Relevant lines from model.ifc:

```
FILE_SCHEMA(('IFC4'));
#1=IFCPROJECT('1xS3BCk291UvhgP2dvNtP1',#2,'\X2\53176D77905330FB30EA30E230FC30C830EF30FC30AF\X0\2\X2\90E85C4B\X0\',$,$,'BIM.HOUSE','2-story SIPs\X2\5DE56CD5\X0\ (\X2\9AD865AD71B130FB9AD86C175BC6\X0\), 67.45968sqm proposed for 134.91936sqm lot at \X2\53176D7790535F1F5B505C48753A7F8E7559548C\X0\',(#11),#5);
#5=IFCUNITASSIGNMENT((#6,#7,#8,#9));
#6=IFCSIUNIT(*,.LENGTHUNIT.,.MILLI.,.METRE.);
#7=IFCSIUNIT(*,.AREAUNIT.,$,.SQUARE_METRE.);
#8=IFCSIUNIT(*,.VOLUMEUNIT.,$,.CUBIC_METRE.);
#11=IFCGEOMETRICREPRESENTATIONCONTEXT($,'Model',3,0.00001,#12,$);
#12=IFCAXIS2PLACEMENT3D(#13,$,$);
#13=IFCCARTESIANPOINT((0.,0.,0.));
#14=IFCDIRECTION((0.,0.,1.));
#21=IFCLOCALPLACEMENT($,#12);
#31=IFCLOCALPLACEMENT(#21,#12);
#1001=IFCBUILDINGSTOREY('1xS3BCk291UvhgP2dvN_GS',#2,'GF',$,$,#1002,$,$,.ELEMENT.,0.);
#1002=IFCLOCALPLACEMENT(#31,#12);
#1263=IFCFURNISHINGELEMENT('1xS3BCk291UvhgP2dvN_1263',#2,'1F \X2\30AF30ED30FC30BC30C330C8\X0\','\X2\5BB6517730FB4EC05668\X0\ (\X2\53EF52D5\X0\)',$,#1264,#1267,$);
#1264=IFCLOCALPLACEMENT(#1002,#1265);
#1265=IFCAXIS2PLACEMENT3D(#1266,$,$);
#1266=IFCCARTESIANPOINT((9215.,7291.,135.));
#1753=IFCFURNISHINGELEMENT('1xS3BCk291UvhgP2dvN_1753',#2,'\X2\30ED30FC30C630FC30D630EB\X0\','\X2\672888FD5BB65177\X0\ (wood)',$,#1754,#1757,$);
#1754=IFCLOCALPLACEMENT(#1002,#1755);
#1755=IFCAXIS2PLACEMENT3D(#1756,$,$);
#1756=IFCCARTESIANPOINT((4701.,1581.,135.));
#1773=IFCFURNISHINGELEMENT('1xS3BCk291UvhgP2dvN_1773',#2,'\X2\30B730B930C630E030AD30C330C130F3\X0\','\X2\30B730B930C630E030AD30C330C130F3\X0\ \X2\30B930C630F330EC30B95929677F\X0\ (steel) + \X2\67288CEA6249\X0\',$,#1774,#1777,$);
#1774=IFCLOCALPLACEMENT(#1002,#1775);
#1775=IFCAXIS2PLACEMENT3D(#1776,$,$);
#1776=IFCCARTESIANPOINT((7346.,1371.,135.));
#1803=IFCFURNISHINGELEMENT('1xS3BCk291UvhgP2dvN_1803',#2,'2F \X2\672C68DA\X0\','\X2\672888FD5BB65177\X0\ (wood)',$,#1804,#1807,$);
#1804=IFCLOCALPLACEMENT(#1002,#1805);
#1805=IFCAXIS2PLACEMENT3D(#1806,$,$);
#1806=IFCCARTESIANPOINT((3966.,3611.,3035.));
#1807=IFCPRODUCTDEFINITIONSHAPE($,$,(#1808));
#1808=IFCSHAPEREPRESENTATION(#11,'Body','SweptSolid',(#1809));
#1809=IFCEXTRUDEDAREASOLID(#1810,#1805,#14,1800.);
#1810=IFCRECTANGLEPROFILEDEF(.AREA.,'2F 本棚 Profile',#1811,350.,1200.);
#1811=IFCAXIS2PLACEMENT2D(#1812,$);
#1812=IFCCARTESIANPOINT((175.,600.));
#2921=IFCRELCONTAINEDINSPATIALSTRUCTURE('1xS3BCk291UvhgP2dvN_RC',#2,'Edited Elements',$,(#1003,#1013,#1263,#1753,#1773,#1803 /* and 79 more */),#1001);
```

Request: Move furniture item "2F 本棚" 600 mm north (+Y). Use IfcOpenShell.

```python
import ifcopenshell
import ifcopenshell.api.geometry
import ifcopenshell.util.placement
import ifcopenshell.util.unit

model = ifcopenshell.open("model.ifc")
unit_scale = ifcopenshell.util.unit.calculate_unit_scale(model)

item = model.by_guid("1xS3BCk291UvhgP2dvN_1803")
matrix = ifcopenshell.util.placement.get_local_placement(item.ObjectPlacement)
matrix[1, 3] += 0.6 / unit_scale
ifcopenshell.api.geometry.edit_object_placement(model, product=item, matrix=matrix, is_si=False)

print(ifcopenshell.util.placement.get_local_placement(item.ObjectPlacement).round(3) + 0.0)

model.write("model_rev.ifc")
```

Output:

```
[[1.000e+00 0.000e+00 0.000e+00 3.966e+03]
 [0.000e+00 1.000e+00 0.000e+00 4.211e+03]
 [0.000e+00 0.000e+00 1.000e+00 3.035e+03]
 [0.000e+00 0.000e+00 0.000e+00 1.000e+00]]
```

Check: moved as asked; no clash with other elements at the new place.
